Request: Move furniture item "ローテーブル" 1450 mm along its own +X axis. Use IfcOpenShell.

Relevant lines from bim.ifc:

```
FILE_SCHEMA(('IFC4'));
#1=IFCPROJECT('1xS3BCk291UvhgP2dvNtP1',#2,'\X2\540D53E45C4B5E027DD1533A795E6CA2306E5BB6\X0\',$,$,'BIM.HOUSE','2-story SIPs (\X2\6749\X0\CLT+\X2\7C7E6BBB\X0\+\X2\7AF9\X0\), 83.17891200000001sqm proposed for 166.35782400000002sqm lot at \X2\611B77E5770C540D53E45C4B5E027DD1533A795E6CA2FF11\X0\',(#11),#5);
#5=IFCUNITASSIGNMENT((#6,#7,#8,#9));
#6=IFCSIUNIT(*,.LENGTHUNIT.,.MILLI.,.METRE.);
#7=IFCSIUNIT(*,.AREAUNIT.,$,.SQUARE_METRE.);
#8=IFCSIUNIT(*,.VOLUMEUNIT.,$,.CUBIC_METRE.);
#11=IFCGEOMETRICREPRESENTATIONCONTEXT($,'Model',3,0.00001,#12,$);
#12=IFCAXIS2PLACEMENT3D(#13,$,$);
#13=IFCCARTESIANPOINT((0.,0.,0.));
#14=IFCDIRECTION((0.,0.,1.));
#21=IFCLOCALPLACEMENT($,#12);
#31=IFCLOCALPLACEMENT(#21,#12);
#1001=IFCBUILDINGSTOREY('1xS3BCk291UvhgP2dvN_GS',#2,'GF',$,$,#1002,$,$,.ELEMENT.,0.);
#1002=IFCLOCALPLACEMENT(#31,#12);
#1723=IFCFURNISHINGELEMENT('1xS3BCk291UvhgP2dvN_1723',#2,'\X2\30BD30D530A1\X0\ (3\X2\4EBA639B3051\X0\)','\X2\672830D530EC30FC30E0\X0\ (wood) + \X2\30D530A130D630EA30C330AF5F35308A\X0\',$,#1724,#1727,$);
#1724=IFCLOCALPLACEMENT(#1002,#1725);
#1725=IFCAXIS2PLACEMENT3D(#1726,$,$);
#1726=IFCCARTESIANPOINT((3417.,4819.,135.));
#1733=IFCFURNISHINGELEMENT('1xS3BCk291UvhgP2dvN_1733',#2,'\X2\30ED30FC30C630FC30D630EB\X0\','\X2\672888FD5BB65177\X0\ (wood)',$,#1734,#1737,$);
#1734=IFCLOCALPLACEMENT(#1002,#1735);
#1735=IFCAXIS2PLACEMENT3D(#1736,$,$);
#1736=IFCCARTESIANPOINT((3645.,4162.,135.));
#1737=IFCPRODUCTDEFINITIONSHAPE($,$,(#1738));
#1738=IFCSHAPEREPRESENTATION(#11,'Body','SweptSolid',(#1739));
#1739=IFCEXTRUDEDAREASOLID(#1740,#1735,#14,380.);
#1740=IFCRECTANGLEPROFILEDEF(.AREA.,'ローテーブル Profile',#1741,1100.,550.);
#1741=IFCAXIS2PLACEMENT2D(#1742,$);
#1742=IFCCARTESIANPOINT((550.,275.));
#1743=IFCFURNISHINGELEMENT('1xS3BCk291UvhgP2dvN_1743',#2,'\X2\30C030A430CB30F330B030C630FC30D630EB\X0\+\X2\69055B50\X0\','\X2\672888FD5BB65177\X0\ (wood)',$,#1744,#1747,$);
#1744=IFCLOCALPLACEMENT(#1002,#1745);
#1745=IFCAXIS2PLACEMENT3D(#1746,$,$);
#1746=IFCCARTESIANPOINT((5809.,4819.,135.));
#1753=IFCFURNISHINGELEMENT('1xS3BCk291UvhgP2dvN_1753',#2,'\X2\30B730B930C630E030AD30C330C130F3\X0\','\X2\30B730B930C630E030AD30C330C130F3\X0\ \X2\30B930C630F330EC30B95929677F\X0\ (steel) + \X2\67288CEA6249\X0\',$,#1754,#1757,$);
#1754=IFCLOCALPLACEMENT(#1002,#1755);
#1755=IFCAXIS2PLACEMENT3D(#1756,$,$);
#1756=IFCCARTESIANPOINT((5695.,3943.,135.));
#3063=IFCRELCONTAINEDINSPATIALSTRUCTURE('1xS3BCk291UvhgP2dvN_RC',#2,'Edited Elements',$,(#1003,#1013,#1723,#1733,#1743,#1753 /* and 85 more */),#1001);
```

```python
import ifcopenshell
import ifcopenshell.api.geometry
import ifcopenshell.util.placement

model = ifcopenshell.open("bim.ifc")

item = model.by_guid("1xS3BCk291UvhgP2dvN_1733")
matrix = ifcopenshell.util.placement.get_local_placement(item.ObjectPlacement)
matrix[:3, 3] += matrix[:3, 0] * 1450.0
ifcopenshell.api.geometry.edit_object_placement(model, product=item, matrix=matrix, is_si=False)

print(ifcopenshell.util.placement.get_local_placement(item.ObjectPlacement).round(3) + 0.0)

model.write("bim_updated.ifc")
```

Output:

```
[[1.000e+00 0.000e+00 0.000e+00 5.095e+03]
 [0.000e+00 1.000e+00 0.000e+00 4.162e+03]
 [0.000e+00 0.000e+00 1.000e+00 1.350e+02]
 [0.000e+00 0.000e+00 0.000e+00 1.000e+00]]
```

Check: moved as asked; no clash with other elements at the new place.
